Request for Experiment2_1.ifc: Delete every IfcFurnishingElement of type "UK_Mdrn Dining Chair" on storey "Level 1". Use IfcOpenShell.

First a look at what the model holds.

```python
import ifcopenshell
import ifcopenshell.util.element

model = ifcopenshell.open("Experiment2_1.ifc")
print(model.schema)
storey = next(s for s in model.by_type("IfcBuildingStorey") if s.Name == "Level 1")
furniture = [e for e in ifcopenshell.util.element.get_decomposition(storey) if e.is_a("IfcFurnishingElement")]
seen = {}
for e in furniture:
    element_type = ifcopenshell.util.element.get_type(e)
    name = element_type.Name if element_type not in (None, e) else None
    seen[name] = seen.get(name, 0) + 1
for name, count in sorted(seen.items(), key=str):
    print(count, "x", name)
```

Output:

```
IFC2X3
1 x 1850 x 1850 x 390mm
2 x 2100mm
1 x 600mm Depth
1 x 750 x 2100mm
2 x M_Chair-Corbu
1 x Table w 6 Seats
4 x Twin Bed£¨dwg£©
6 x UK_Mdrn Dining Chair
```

```python
import ifcopenshell
import ifcopenshell.api.root
import ifcopenshell.util.element

model = ifcopenshell.open("Experiment2_1.ifc")

storey = next(s for s in model.by_type("IfcBuildingStorey") if s.Name == "Level 1")
furniture = [e for e in ifcopenshell.util.element.get_decomposition(storey) if e.is_a("IfcFurnishingElement")]
targets = [e for e in furniture if (t := ifcopenshell.util.element.get_type(e)) not in (None, e) and t.Name == "UK_Mdrn Dining Chair"]

for e in targets:
    ifcopenshell.api.root.remove_product(model, product=e)
print(len(targets), "removed")

model.write("Experiment2_1_edited.ifc")
```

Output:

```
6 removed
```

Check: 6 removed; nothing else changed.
